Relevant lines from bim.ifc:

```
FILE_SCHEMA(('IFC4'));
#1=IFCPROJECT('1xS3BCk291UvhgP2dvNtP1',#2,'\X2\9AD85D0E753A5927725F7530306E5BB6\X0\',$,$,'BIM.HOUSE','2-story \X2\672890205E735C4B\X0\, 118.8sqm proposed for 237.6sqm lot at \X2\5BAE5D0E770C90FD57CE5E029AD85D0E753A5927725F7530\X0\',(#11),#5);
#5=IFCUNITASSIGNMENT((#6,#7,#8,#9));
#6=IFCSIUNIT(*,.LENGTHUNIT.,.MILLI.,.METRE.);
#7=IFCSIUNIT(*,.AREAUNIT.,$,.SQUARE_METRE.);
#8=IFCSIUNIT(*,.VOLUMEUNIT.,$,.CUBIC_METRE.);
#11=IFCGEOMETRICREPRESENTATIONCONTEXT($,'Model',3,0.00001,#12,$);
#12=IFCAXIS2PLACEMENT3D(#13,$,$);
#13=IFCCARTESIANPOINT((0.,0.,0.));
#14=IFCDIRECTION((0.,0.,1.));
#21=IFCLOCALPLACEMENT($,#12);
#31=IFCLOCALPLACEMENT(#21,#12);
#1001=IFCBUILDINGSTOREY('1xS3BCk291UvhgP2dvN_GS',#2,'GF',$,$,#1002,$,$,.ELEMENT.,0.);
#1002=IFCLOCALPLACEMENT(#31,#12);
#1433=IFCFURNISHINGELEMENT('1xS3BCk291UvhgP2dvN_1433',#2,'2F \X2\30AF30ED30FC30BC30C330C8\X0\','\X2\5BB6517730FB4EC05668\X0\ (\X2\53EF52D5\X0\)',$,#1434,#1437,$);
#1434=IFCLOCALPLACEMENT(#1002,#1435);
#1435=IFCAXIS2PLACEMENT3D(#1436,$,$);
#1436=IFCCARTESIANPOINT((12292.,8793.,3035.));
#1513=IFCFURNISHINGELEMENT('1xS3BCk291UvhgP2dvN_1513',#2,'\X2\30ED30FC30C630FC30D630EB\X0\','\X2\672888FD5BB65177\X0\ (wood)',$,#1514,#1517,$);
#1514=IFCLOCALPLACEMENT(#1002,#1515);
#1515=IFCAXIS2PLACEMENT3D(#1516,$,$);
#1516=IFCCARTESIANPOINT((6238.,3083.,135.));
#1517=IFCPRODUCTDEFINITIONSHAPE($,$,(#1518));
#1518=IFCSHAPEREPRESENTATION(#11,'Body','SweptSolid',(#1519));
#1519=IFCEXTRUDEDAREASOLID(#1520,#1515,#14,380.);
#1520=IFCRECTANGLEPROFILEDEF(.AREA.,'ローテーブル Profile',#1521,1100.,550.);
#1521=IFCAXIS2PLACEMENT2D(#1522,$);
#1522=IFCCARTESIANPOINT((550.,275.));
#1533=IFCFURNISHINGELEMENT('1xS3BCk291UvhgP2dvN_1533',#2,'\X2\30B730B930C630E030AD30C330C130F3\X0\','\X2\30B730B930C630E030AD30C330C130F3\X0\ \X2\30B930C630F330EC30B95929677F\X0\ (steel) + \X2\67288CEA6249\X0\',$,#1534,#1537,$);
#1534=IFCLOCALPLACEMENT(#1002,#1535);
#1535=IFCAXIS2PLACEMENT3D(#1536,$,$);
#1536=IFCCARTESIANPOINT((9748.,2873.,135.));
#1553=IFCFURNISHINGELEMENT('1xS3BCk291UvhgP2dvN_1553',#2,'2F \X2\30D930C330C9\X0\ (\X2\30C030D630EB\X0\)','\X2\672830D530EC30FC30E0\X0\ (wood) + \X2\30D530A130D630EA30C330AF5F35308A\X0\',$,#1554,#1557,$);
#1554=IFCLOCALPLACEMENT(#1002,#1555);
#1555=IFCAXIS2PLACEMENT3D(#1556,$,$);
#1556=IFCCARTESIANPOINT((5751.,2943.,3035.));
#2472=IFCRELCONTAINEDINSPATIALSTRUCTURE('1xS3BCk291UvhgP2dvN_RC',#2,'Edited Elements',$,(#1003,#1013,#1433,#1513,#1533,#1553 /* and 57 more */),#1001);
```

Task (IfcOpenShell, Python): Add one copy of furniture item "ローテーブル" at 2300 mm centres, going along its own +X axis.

```python
import ifcopenshell
import ifcopenshell.api.geometry
import ifcopenshell.api.root
import ifcopenshell.util.element
import ifcopenshell.util.placement
import ifcopenshell.util.unit

model = ifcopenshell.open("bim.ifc")
unit_scale = ifcopenshell.util.unit.calculate_unit_scale(model)


def reuse_history(source, copy):
    """copy_class also copies each property set's owner history, people and application; keep the originals."""
    for rel in copy.IsDefinedBy:
        if rel.is_a("IfcRelDefinesByProperties") and (history := rel.RelatingPropertyDefinition.OwnerHistory):
            rel.RelatingPropertyDefinition.OwnerHistory = source.OwnerHistory
            ifcopenshell.util.element.remove_deep2(model, history)


source = model.by_guid("1xS3BCk291UvhgP2dvN_1513")
base = ifcopenshell.util.placement.get_local_placement(source.ObjectPlacement)
step = base[:3, 0] * 2.3 / unit_scale

for i in range(1, 2):
    copy = ifcopenshell.api.root.copy_class(model, product=source)
    copy.Representation = ifcopenshell.util.element.copy_deep(
        model, source.Representation, exclude=["IfcGeometricRepresentationContext", "IfcRepresentationMap"]
    )
    reuse_history(source, copy)
    matrix = base.copy()
    matrix[:3, 3] += i * step
    print("added at", matrix[:3, 3].round(3) + 0.0)
    ifcopenshell.api.geometry.edit_object_placement(model, product=copy, matrix=matrix, is_si=False)

model.write("bim_v2.ifc")
```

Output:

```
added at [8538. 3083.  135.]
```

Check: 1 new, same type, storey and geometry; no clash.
